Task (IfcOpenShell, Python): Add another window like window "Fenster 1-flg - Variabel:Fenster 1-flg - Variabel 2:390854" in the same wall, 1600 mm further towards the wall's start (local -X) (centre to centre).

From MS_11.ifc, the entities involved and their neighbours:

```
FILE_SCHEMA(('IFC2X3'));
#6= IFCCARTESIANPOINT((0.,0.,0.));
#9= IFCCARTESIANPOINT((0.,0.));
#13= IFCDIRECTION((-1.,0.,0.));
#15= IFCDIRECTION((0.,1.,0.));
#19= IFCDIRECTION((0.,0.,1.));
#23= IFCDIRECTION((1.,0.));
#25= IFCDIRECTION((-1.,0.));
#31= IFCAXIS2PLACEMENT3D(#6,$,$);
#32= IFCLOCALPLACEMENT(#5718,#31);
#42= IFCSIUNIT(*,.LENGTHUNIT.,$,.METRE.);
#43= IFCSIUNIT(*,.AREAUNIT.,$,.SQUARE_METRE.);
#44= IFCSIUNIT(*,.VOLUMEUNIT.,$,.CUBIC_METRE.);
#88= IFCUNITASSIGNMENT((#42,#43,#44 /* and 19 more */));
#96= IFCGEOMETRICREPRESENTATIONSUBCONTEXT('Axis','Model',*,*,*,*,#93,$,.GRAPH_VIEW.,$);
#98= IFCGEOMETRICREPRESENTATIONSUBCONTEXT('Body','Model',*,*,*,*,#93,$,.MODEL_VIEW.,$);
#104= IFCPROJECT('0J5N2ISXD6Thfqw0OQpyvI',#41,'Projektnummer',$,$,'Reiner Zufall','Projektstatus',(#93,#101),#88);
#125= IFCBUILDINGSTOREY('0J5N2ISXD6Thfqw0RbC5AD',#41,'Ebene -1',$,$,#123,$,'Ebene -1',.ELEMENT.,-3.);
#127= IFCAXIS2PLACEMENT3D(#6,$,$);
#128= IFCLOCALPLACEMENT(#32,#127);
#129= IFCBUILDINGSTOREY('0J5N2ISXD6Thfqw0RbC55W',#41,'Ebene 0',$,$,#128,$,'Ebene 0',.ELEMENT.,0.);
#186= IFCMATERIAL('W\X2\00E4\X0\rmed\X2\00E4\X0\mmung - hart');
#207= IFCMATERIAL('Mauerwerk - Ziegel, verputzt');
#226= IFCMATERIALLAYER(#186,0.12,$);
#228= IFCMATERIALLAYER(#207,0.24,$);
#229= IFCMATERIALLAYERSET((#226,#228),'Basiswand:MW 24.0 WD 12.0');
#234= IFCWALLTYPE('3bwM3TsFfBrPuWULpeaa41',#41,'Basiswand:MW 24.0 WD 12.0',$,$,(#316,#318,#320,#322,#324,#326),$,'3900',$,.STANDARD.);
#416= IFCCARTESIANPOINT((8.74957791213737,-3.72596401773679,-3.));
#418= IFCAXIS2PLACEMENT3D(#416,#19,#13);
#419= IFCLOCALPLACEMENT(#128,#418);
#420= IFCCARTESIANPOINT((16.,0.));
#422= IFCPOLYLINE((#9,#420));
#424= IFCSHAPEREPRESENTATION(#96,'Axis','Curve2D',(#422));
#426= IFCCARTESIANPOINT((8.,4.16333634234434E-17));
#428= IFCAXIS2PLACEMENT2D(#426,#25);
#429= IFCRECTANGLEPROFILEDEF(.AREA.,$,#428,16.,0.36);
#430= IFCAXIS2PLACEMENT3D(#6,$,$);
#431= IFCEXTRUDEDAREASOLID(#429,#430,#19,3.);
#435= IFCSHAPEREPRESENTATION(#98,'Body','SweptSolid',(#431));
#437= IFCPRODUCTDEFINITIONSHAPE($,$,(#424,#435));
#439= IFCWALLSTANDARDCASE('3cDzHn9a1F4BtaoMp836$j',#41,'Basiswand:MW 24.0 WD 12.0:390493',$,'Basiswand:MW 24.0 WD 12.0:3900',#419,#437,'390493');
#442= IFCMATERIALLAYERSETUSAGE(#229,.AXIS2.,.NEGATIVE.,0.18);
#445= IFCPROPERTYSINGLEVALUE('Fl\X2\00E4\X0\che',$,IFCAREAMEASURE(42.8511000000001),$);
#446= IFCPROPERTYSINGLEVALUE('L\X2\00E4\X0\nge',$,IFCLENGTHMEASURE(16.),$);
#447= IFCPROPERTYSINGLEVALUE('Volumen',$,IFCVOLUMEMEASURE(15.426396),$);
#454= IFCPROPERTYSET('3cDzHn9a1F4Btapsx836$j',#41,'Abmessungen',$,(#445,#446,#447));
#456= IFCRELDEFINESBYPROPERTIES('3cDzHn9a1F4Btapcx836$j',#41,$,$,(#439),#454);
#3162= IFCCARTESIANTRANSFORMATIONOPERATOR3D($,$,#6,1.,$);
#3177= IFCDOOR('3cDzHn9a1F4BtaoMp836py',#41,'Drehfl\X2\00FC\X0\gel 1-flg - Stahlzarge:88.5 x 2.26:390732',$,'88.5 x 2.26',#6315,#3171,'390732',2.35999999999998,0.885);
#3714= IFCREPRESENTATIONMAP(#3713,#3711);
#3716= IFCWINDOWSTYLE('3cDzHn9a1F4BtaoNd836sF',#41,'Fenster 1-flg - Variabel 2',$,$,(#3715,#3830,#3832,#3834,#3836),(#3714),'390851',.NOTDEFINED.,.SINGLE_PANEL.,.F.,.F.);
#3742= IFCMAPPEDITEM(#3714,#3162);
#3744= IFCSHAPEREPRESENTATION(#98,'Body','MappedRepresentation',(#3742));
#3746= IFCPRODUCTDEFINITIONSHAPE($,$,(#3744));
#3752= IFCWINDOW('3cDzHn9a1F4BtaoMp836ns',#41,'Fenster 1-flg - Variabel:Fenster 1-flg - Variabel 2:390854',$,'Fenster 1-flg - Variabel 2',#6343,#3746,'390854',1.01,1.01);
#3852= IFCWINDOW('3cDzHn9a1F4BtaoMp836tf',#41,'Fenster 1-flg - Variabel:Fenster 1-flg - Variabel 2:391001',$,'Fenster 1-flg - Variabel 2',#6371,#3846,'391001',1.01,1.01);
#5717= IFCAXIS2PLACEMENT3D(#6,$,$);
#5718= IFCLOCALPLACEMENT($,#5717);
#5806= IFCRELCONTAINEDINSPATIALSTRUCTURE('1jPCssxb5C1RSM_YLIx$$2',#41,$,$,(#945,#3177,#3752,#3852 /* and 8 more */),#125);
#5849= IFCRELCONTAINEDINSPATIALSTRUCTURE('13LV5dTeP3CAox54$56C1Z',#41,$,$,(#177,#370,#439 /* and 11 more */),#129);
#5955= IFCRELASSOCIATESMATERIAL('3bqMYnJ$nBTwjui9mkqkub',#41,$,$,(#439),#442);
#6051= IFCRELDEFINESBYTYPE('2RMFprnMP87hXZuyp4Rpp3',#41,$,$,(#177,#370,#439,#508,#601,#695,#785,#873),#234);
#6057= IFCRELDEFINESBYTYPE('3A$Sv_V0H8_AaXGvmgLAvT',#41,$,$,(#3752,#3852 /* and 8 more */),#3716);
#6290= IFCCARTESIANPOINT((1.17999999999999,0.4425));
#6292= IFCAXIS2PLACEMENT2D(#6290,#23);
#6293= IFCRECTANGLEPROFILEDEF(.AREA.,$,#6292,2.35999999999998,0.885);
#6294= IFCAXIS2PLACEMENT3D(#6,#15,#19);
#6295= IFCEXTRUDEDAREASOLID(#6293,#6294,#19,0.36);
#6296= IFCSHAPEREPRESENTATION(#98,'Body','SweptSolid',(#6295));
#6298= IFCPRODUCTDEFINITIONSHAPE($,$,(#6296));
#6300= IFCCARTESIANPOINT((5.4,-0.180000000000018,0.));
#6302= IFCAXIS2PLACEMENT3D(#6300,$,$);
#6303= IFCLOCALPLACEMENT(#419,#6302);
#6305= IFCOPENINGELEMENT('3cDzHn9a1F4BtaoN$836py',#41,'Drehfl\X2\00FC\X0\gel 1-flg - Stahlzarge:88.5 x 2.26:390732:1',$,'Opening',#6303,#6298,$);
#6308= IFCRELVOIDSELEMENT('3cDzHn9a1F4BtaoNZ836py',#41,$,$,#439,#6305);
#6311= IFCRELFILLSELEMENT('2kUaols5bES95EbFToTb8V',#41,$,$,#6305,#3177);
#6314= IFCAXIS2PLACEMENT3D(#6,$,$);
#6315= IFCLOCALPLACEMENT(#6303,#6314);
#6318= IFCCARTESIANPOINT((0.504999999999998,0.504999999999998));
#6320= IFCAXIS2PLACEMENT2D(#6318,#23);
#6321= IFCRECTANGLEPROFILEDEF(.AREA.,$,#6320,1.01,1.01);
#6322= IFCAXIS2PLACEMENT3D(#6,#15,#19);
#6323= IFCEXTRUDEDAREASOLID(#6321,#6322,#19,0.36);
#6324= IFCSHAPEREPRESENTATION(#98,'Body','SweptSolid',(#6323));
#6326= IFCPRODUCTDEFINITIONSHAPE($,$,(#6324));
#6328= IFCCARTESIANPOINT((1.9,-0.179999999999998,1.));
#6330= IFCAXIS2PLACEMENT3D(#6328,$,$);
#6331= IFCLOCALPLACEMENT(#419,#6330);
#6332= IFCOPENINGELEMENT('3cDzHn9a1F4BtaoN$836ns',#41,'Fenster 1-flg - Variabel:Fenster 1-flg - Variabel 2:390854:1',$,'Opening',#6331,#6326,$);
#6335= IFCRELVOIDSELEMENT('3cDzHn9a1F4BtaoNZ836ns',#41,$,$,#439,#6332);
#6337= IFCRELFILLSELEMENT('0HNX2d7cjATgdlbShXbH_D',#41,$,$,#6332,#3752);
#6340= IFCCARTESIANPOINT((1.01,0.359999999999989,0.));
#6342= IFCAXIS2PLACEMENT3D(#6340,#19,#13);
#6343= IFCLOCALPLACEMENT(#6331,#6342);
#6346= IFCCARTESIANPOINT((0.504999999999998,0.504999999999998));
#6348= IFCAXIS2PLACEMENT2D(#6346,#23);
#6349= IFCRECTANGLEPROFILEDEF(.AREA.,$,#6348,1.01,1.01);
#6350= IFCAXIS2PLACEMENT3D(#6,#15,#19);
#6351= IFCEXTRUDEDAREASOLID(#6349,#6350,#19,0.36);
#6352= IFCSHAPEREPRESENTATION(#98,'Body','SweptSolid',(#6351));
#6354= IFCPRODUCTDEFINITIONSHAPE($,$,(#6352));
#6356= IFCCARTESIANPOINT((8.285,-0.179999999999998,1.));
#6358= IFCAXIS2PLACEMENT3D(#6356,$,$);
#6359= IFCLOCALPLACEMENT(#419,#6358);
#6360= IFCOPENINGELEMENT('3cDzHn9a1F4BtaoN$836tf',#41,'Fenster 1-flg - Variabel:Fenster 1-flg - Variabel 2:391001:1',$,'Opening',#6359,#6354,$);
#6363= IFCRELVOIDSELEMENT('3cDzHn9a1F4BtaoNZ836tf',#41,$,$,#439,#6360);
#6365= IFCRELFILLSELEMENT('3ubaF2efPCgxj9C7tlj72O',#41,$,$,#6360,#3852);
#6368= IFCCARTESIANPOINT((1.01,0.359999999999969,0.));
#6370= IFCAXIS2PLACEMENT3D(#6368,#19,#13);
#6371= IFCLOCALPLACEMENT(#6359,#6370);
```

```python
import ifcopenshell
import ifcopenshell.api.feature
import ifcopenshell.api.geometry
import ifcopenshell.api.pset
import ifcopenshell.api.root
import ifcopenshell.geom
import ifcopenshell.util.element
import ifcopenshell.util.placement
import ifcopenshell.util.shape
import ifcopenshell.util.unit

model = ifcopenshell.open("MS_11.ifc")
area_scale = ifcopenshell.util.unit.calculate_unit_scale(model, "AREAUNIT")
volume_scale = ifcopenshell.util.unit.calculate_unit_scale(model, "VOLUMEUNIT")
settings = ifcopenshell.geom.settings()


def volume(element):
    """Net volume in cubic metres, openings subtracted."""
    shape = ifcopenshell.geom.create_shape(settings, element)
    return ifcopenshell.util.shape.get_volume(shape.geometry)


def reuse_history(source, copy):
    """copy_class also copies each property set's owner history, people and application; keep the originals."""
    for rel in copy.IsDefinedBy:
        if rel.is_a("IfcRelDefinesByProperties") and (history := rel.RelatingPropertyDefinition.OwnerHistory):
            rel.RelatingPropertyDefinition.OwnerHistory = source.OwnerHistory
            ifcopenshell.util.element.remove_deep2(model, history)


window = model.by_id(3752)
opening = window.FillsVoids[0].RelatingOpeningElement
wall = opening.VoidsElements[0].RelatingBuildingElement
before = volume(wall)
shift = ifcopenshell.util.placement.get_local_placement(wall.ObjectPlacement)[:3, 0] * -1.6

# copy_class copies the void relationship, type, container and properties, but no geometry.
new_opening = ifcopenshell.api.root.copy_class(model, product=opening)
new_opening.Representation = ifcopenshell.util.element.copy_deep(
    model, opening.Representation, exclude=["IfcGeometricRepresentationContext", "IfcRepresentationMap"]
)
new_opening.Name = "Fenster 1-flg - Variabel:Fenster 1-flg - Variabel 2"
new_window = ifcopenshell.api.root.copy_class(model, product=window)
new_window.Representation = ifcopenshell.util.element.copy_deep(
    model, window.Representation, exclude=["IfcGeometricRepresentationContext", "IfcRepresentationMap"]
)
new_window.Name = "Fenster 1-flg - Variabel:Fenster 1-flg - Variabel 2"
new_window.Tag = None
reuse_history(window, new_window)
fills = ifcopenshell.api.feature.add_filling(model, opening=new_opening, element=new_window)
fills.OwnerHistory = new_window.OwnerHistory  # required in IFC2X3

for old, new in ((opening, new_opening), (window, new_window)):
    matrix = ifcopenshell.util.placement.get_local_placement(old.ObjectPlacement)
    matrix[:3, 3] += shift
    ifcopenshell.api.geometry.edit_object_placement(model, product=new, matrix=matrix, is_si=False)

after = volume(wall)
thickness = 0.36  # wall thickness in metres

# Update the wall's stored quantities.
pset = model.by_id(ifcopenshell.util.element.get_pset(wall, "Abmessungen", should_inherit=False)["id"])
ifcopenshell.api.pset.edit_pset(model, pset=pset, properties={
    "Fläche": model.create_entity("IfcAreaMeasure", after / thickness / area_scale),
    "Volumen": model.create_entity("IfcVolumeMeasure", after / volume_scale),
})

print(f"wall volume {before:.3f} -> {after:.3f} m3")

model.write("MS_11_edited.ifc")
```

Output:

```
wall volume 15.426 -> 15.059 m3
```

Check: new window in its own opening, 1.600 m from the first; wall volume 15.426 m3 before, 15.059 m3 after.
